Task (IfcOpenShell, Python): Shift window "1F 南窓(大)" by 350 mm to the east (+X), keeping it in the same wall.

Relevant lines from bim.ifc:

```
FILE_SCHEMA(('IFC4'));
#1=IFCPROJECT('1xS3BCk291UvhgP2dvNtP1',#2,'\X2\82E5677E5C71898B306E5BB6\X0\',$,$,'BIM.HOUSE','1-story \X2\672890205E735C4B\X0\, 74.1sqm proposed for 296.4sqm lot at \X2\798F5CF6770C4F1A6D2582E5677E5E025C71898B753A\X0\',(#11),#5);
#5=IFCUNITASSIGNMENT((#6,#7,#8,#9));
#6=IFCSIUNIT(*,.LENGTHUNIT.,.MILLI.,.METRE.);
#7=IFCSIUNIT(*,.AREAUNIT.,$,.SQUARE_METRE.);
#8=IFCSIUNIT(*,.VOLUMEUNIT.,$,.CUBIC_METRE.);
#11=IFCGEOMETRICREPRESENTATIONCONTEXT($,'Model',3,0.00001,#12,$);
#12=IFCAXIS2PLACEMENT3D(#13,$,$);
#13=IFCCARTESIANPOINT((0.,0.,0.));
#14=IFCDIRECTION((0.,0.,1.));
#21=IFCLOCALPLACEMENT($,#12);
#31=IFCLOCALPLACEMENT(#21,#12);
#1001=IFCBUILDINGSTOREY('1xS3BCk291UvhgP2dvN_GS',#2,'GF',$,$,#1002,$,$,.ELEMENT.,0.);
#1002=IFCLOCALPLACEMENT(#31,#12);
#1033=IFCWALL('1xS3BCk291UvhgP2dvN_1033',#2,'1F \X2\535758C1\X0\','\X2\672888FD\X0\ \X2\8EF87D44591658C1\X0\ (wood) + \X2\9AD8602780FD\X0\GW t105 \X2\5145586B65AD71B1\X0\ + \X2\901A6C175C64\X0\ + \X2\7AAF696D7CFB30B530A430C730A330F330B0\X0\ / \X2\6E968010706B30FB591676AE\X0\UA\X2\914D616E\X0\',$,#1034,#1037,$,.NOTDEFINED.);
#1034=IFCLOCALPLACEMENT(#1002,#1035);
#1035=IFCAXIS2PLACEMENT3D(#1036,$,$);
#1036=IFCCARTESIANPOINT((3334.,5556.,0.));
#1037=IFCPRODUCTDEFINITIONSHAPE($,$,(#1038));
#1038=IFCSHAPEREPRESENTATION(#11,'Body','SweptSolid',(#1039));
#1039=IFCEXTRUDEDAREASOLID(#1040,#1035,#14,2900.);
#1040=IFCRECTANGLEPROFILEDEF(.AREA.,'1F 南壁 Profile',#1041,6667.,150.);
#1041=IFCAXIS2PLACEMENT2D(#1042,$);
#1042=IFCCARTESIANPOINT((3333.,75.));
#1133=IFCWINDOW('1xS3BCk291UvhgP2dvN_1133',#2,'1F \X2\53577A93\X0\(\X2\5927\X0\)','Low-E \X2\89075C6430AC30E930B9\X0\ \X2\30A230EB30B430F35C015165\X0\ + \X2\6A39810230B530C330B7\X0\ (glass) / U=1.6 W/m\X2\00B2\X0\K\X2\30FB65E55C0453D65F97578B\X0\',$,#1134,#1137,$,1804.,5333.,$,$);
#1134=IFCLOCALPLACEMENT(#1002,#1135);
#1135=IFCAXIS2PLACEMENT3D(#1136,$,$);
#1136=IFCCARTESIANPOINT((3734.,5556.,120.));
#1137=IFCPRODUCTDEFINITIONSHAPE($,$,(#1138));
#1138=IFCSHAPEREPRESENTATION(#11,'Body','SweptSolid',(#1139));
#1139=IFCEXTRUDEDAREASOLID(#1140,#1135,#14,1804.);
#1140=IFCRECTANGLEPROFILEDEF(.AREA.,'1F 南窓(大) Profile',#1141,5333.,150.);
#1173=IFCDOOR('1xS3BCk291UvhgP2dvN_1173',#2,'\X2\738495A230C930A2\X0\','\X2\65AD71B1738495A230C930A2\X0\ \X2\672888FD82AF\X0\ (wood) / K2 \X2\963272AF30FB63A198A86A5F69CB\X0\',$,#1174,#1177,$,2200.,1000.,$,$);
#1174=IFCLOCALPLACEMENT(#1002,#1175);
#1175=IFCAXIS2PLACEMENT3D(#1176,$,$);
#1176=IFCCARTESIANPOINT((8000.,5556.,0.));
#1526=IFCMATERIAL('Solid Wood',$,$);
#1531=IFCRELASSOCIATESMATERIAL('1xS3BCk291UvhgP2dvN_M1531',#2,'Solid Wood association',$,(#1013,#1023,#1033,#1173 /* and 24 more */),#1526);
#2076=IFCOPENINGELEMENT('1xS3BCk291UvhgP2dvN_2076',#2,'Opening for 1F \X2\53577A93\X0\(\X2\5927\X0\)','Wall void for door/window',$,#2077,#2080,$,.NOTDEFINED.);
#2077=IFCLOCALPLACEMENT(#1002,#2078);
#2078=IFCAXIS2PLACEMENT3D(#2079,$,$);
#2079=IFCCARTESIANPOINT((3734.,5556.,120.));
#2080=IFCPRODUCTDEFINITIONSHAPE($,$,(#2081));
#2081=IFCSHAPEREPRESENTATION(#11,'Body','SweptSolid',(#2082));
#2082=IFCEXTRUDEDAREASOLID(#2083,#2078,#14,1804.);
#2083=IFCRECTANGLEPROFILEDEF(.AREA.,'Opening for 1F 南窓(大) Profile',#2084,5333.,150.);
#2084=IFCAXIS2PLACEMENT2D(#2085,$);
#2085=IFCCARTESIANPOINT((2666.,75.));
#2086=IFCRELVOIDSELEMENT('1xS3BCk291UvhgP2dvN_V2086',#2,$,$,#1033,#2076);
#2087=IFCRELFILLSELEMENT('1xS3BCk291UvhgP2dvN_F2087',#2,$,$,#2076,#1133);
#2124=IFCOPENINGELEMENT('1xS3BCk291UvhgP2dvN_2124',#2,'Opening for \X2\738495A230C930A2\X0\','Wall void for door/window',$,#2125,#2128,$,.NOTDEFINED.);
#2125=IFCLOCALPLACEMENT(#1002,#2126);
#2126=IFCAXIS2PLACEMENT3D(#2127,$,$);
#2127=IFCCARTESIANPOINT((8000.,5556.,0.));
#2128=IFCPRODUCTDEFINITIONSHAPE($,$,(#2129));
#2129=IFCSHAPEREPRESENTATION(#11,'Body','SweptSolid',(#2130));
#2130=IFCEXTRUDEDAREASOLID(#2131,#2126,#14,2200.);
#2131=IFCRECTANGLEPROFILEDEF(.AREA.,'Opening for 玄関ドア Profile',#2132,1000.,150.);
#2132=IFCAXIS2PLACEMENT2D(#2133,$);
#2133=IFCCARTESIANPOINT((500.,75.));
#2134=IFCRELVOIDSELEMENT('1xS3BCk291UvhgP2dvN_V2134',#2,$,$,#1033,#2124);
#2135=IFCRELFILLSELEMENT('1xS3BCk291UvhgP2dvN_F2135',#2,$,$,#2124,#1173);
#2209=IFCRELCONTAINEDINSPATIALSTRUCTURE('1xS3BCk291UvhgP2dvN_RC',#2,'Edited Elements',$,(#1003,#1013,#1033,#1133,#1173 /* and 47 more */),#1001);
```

```python
import ifcopenshell
import ifcopenshell.api.geometry
import ifcopenshell.util.placement
import ifcopenshell.util.unit

model = ifcopenshell.open("bim.ifc")
unit_scale = ifcopenshell.util.unit.calculate_unit_scale(model)

window = model.by_guid("1xS3BCk291UvhgP2dvN_1133")
opening = window.FillsVoids[0].RelatingOpeningElement
wall = opening.VoidsElements[0].RelatingBuildingElement

wall_matrix = ifcopenshell.util.placement.get_local_placement(wall.ObjectPlacement)
shift = wall_matrix[:3, 0] * 0.35 / unit_scale
before = ifcopenshell.util.placement.get_local_placement(window.ObjectPlacement)[:3, 3].copy()

# The window is not placed relative to its opening, so move both.
for product in (opening, window):
    matrix = ifcopenshell.util.placement.get_local_placement(product.ObjectPlacement)
    matrix[:3, 3] += shift
    ifcopenshell.api.geometry.edit_object_placement(model, product=product, matrix=matrix, is_si=False)

after = ifcopenshell.util.placement.get_local_placement(window.ObjectPlacement)[:3, 3]
print("window moved by", (after - before).round(3) + 0.0)

model.write("bim_v2.ifc")
```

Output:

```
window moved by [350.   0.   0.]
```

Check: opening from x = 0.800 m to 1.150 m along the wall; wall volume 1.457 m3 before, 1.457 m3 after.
